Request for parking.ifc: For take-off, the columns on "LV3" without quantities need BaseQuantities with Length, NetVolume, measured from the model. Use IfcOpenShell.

First a look at what the model holds.

```python
import ifcopenshell
import ifcopenshell.util.element
import ifcopenshell.util.unit

model = ifcopenshell.open("parking.ifc")
print(model.schema)
for unit_type in ("LENGTHUNIT", "AREAUNIT", "VOLUMEUNIT"):
    print(unit_type, ifcopenshell.util.unit.calculate_unit_scale(model, unit_type))
storey = next(s for s in model.by_type("IfcBuildingStorey") if s.Name == "LV3")
columns = [e for e in ifcopenshell.util.element.get_decomposition(storey) if e.is_a("IfcColumn")]
for e in sorted(columns, key=lambda e: e.id()):
    print(e.id(), e.is_a(), e.Name, list(ifcopenshell.util.element.get_psets(e, qtos_only=True)), sep=" | ")
```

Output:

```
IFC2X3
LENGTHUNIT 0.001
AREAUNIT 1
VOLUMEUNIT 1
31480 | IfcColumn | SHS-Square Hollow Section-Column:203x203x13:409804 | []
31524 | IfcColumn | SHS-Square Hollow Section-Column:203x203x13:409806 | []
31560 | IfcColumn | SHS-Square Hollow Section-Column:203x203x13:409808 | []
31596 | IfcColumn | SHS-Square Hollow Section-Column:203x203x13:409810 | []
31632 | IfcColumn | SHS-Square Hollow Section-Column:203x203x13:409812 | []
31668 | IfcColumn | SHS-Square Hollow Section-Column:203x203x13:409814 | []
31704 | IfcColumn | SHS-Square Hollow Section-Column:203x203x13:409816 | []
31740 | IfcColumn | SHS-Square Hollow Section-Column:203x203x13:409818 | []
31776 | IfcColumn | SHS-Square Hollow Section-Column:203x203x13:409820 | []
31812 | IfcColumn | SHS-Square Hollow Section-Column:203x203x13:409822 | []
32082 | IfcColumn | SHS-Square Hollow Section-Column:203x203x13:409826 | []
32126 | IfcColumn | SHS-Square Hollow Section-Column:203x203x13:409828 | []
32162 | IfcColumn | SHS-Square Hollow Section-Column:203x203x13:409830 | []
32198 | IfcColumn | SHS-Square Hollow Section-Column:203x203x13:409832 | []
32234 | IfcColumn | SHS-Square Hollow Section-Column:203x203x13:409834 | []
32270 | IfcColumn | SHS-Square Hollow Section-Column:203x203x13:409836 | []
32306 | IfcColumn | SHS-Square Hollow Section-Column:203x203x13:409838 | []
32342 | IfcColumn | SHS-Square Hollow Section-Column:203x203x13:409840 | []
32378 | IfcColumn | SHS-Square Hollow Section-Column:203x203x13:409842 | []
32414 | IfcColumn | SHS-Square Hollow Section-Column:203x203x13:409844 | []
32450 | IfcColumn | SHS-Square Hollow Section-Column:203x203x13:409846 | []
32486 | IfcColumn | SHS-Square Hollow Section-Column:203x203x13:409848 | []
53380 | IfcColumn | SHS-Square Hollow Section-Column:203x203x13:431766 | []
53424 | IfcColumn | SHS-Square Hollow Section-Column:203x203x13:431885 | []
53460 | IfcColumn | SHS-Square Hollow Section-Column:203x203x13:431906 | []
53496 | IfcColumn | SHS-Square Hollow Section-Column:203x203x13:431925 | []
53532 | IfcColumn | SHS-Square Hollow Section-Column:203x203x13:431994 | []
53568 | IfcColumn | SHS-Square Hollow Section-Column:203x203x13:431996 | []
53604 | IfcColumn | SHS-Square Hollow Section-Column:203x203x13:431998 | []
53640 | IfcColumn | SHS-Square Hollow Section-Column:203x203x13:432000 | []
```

```python
import ifcopenshell
import ifcopenshell.api.pset
import ifcopenshell.geom
import ifcopenshell.util.element
import ifcopenshell.util.shape
import ifcopenshell.util.unit

model = ifcopenshell.open("parking.ifc")
unit_scale = ifcopenshell.util.unit.calculate_unit_scale(model)
volume_scale = ifcopenshell.util.unit.calculate_unit_scale(model, "VOLUMEUNIT")
settings = ifcopenshell.geom.settings()

storey = next(s for s in model.by_type("IfcBuildingStorey") if s.Name == "LV3")
columns = [e for e in ifcopenshell.util.element.get_decomposition(storey) if e.is_a("IfcColumn")]

for e in sorted(columns, key=lambda e: e.id()):
    if ifcopenshell.util.element.get_psets(e, qtos_only=True, should_inherit=False):
        continue
    # Geometry comes back in metres, in the element's own axes.
    shape = ifcopenshell.geom.create_shape(settings, e)
    values = {
        "Length": ifcopenshell.util.shape.get_z(shape.geometry) / unit_scale,
        "NetVolume": ifcopenshell.util.shape.get_volume(shape.geometry) / volume_scale,
    }
    qto = ifcopenshell.api.pset.add_qto(model, product=e, name="BaseQuantities")
    ifcopenshell.api.pset.edit_qto(model, qto=qto, properties=values)
    print(e.id(), {k: round(v, 3) for k, v in values.items()})

model.write("parking_rev.ifc")
```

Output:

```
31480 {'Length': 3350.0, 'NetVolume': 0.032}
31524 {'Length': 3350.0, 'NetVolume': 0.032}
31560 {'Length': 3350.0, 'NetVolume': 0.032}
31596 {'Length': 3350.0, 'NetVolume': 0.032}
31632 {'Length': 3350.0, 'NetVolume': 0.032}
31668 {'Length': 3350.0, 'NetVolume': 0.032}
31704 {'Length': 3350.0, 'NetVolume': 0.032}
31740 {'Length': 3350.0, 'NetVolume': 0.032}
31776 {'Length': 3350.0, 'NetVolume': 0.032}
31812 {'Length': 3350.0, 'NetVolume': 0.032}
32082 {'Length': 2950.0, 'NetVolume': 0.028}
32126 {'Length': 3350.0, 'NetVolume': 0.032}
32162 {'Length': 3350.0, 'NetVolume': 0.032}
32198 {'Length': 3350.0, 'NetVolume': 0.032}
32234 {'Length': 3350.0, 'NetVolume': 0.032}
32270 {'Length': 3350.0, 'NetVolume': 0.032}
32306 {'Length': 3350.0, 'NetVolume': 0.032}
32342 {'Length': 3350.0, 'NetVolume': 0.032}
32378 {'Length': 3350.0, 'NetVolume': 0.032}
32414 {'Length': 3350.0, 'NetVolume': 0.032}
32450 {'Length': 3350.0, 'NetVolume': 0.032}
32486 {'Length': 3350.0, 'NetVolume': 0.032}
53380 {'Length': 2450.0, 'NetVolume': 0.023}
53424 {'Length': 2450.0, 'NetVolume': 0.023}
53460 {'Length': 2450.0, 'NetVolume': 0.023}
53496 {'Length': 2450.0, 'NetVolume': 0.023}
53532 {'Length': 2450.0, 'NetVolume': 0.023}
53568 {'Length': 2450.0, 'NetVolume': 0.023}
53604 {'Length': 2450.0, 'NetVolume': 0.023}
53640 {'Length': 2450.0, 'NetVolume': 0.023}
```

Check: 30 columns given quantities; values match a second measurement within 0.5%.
